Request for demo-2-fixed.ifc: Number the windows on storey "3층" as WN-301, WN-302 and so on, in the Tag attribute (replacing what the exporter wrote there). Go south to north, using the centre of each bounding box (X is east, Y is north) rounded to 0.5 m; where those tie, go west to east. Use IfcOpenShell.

First a look at what the model holds.

```python
import ifcopenshell
import ifcopenshell.util.element
import ifcopenshell.util.placement

model = ifcopenshell.open("demo-2-fixed.ifc")
print(model.schema)
storey = next(s for s in model.by_type("IfcBuildingStorey") if s.Name == "3층")
windows = [e for e in ifcopenshell.util.element.get_decomposition(storey) if e.is_a("IfcWindow")]
for e in sorted(windows, key=lambda e: e.id()):
    origin = ifcopenshell.util.placement.get_local_placement(e.ObjectPlacement)[:3, 3]
    print(e.id(), e.Tag, e.Name, origin.round(2) + 0.0, sep=" | ")
```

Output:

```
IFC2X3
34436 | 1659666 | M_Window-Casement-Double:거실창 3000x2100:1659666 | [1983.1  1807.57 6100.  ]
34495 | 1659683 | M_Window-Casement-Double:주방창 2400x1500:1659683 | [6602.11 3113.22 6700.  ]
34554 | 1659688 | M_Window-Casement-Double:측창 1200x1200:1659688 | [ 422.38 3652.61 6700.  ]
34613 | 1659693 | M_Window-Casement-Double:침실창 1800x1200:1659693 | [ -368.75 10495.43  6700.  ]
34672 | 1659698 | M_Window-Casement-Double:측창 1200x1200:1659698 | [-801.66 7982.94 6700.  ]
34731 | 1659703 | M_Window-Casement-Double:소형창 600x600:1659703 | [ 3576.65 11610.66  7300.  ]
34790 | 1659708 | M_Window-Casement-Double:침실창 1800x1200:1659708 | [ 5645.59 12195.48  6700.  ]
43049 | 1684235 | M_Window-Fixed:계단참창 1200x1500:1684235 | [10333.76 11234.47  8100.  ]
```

```python
import ifcopenshell
import ifcopenshell.geom
import ifcopenshell.util.element
import ifcopenshell.util.shape

model = ifcopenshell.open("demo-2-fixed.ifc")
settings = ifcopenshell.geom.settings()
settings.set("use-world-coords", True)


def centre(element):
    shape = ifcopenshell.geom.create_shape(settings, element)
    return ifcopenshell.util.shape.get_bbox_centroid(shape.geometry)


storey = next(s for s in model.by_type("IfcBuildingStorey") if s.Name == "3층")
windows = [e for e in ifcopenshell.util.element.get_decomposition(storey) if e.is_a("IfcWindow")]

# Insertion points can sit at a corner or the storey origin, so sort by the geometry (in metres).
centres = {e: centre(e) for e in windows}
windows.sort(key=lambda e: (round(centres[e][1] / 0.5), centres[e][0]))

for i, e in enumerate(windows, start=1):
    number = f"WN-3{i:02d}"
    e.Tag = number
    print(e.id(), number)

model.write("demo-2-fixed_rev.ifc")
```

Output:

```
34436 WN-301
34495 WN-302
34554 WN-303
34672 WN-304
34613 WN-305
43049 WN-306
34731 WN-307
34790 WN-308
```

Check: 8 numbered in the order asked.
